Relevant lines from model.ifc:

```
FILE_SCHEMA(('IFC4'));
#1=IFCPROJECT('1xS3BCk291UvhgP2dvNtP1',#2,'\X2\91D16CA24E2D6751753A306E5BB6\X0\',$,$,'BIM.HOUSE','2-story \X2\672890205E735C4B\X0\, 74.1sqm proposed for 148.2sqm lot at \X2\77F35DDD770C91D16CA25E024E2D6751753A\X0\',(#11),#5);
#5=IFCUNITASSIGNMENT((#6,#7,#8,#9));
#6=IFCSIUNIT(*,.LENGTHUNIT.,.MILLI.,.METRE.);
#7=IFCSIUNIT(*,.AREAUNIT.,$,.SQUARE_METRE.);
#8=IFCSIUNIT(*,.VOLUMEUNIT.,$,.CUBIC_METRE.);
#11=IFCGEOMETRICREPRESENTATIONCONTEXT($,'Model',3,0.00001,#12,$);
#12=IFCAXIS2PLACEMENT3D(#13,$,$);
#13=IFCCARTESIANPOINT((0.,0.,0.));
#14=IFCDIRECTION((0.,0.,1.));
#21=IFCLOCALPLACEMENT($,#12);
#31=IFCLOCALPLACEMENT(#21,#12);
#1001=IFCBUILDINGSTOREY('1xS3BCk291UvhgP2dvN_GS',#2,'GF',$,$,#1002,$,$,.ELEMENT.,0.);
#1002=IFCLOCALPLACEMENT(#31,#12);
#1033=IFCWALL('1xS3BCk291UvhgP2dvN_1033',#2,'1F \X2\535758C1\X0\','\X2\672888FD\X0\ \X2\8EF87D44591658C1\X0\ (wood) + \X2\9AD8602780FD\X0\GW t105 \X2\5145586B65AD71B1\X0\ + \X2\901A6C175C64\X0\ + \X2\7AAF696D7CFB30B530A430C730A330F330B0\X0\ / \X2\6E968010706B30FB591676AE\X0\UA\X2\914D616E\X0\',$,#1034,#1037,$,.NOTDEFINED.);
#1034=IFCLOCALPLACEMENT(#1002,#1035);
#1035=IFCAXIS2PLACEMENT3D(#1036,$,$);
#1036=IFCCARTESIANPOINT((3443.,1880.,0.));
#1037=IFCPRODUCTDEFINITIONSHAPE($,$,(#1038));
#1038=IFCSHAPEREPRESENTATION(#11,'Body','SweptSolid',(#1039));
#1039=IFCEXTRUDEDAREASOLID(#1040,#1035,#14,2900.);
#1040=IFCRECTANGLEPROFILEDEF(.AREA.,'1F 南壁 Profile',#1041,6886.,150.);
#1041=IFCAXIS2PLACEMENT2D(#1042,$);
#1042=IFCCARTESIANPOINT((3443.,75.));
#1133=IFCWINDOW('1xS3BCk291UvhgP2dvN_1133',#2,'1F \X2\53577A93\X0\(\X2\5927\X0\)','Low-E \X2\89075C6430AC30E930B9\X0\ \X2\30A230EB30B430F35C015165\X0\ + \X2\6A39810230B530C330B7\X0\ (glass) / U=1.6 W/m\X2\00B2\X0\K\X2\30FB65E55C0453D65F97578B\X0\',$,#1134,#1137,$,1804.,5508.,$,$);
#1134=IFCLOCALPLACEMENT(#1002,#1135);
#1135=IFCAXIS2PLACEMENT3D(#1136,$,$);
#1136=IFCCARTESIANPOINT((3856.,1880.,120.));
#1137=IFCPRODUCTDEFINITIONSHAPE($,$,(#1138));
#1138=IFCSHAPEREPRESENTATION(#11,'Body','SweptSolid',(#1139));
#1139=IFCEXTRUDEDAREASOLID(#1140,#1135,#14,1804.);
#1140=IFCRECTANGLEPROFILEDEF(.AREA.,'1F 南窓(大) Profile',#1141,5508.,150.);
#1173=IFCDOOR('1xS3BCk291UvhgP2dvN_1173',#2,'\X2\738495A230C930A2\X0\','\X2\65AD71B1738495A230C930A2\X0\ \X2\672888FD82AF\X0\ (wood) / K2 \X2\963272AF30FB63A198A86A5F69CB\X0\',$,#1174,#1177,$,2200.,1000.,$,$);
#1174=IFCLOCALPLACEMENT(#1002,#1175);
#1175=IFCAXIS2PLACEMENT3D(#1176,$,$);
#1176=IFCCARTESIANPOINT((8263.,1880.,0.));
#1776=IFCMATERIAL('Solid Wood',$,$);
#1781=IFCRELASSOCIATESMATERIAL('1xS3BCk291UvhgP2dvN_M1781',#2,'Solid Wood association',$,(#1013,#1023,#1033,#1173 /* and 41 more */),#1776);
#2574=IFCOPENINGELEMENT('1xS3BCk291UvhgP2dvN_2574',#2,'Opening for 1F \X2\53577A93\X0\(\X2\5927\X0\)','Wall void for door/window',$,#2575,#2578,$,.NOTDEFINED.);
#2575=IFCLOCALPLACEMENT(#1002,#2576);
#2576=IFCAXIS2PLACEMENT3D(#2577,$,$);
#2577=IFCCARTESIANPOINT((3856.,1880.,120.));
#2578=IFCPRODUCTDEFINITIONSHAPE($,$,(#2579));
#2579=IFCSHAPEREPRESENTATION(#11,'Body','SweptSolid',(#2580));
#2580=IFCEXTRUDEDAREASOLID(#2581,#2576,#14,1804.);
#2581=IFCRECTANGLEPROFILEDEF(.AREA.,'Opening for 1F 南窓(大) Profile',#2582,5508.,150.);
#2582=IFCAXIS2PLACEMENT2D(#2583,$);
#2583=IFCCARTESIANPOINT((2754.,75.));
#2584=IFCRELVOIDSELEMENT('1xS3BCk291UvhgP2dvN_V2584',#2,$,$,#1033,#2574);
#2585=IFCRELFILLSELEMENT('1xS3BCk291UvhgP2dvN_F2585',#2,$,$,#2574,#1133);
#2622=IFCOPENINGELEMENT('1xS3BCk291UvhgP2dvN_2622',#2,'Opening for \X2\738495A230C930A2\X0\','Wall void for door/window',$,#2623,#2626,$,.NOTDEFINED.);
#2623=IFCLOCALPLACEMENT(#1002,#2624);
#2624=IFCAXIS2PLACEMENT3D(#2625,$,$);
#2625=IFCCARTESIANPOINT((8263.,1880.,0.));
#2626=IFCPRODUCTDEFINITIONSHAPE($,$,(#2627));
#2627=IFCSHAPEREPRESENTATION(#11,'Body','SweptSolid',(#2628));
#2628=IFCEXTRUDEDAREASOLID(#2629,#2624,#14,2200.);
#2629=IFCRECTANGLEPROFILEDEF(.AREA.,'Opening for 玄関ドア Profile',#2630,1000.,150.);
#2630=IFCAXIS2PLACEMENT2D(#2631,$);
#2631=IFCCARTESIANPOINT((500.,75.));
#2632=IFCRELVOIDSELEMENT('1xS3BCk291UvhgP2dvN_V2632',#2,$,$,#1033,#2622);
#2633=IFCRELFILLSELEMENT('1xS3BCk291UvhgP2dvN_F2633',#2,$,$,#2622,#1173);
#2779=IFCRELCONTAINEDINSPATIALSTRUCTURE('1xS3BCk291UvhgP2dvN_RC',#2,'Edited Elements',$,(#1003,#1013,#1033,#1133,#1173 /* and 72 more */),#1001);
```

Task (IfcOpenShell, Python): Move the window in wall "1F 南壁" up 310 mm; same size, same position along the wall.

```python
import numpy as np
import ifcopenshell
import ifcopenshell.api.geometry
import ifcopenshell.util.placement
import ifcopenshell.util.unit

model = ifcopenshell.open("model.ifc")
unit_scale = ifcopenshell.util.unit.calculate_unit_scale(model)

window = model.by_id(1133)
opening = window.FillsVoids[0].RelatingOpeningElement
dz = 310.0

shift = np.array([0.0, 0.0, dz])
# The window is not placed relative to its opening, so move both.
for product in (opening, window):
    matrix = ifcopenshell.util.placement.get_local_placement(product.ObjectPlacement)
    matrix[:3, 3] += shift
    ifcopenshell.api.geometry.edit_object_placement(model, product=product, matrix=matrix, is_si=False)

print(f"moved by {dz * unit_scale:+.3f} m")

model.write("model_rev.ifc")
```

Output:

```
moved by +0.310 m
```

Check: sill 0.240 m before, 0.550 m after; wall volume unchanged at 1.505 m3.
